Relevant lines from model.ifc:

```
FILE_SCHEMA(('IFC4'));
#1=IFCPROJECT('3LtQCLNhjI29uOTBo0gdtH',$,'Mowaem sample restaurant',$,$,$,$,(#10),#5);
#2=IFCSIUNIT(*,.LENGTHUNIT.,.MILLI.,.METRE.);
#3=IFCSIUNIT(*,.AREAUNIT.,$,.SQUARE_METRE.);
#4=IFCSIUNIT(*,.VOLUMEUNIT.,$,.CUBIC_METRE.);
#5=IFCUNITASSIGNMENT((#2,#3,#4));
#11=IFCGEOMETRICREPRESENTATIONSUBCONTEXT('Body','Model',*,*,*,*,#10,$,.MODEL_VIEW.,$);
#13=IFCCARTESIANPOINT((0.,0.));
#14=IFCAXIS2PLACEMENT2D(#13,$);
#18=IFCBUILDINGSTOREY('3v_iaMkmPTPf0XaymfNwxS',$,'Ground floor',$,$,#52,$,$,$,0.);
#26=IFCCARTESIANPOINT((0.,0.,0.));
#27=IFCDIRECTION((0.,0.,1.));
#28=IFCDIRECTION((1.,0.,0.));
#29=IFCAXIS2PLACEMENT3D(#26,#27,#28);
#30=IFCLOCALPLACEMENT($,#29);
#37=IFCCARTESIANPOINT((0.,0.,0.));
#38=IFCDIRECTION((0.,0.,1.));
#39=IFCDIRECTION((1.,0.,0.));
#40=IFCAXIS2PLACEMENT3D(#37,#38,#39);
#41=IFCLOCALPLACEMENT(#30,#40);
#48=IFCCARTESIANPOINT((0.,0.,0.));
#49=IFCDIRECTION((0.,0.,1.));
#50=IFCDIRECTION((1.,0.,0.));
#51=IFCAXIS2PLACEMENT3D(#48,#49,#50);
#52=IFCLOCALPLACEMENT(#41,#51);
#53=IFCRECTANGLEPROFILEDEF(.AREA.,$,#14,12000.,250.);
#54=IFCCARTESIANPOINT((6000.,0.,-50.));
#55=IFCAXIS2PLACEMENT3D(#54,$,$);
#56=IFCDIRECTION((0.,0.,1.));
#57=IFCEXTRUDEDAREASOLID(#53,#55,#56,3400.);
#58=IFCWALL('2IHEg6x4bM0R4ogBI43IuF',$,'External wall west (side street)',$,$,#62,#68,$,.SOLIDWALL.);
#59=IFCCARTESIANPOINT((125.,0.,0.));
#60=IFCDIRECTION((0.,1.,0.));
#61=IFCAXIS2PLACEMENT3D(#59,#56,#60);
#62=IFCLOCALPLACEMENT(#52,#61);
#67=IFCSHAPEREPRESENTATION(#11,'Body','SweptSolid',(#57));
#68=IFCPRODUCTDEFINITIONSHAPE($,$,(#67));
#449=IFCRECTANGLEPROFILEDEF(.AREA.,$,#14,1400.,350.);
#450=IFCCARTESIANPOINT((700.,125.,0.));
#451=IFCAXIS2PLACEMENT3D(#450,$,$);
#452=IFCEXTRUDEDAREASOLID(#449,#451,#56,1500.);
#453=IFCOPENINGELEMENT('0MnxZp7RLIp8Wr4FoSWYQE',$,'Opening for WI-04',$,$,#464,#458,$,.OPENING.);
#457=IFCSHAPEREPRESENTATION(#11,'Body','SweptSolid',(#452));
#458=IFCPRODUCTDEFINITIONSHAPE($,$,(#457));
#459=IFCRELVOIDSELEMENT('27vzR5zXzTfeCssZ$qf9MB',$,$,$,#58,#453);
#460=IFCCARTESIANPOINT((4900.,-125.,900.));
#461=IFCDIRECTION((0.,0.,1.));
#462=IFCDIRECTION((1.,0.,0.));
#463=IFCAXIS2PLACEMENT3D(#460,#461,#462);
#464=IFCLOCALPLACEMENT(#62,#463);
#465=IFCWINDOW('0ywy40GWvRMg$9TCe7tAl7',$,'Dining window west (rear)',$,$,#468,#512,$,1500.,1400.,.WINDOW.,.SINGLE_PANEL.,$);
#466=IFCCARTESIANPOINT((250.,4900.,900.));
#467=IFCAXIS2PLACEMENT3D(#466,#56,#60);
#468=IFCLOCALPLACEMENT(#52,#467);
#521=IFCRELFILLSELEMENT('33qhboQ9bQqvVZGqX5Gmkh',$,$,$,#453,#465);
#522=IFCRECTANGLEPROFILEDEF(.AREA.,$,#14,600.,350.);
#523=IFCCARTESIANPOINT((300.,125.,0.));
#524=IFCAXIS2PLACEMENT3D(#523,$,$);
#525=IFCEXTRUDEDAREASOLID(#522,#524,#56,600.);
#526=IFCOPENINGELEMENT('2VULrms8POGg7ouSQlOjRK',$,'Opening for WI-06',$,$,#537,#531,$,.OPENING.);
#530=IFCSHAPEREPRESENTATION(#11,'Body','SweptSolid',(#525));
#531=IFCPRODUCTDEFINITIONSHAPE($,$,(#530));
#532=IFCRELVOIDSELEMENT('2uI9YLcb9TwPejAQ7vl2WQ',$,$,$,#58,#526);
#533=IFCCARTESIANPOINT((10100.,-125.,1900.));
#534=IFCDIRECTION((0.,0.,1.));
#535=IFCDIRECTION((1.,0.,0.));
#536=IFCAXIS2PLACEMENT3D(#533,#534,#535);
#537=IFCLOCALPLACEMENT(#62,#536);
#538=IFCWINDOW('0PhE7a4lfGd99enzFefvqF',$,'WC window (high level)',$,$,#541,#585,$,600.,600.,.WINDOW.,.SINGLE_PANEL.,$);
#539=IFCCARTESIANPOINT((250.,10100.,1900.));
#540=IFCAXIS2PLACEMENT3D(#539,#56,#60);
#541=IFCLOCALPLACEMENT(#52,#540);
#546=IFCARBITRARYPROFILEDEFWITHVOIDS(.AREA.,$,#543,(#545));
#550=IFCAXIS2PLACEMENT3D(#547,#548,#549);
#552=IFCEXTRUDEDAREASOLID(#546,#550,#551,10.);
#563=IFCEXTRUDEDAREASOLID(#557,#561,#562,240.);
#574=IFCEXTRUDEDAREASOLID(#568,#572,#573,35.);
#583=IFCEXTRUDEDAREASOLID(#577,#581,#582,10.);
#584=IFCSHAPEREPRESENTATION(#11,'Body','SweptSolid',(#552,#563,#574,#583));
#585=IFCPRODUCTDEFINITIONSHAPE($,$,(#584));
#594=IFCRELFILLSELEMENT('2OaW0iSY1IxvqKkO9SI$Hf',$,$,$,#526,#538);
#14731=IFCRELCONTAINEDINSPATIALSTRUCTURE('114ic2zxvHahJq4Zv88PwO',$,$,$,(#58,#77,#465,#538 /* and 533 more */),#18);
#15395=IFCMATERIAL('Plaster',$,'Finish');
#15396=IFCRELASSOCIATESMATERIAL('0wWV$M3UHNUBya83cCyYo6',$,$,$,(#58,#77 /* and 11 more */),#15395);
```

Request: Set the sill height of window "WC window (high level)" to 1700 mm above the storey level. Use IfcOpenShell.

```python
import numpy as np
import ifcopenshell
import ifcopenshell.api.geometry
import ifcopenshell.geom
import ifcopenshell.util.element
import ifcopenshell.util.placement
import ifcopenshell.util.shape
import ifcopenshell.util.unit

model = ifcopenshell.open("model.ifc")
unit_scale = ifcopenshell.util.unit.calculate_unit_scale(model)

window = model.by_guid("0PhE7a4lfGd99enzFefvqF")
opening = window.FillsVoids[0].RelatingOpeningElement
storey = ifcopenshell.util.element.get_container(window, ifc_class="IfcBuildingStorey")
level = ifcopenshell.util.placement.get_local_placement(storey.ObjectPlacement)[2, 3]

# The opening's origin need not be at the sill, so measure its lowest point.
shape = ifcopenshell.geom.create_shape(ifcopenshell.geom.settings(), opening)
bottom = ifcopenshell.util.shape.get_shape_bottom_elevation(shape, shape.geometry) / unit_scale
dz = level + 1.7 / unit_scale - bottom

shift = np.array([0.0, 0.0, dz])
# The window is not placed relative to its opening, so move both.
for product in (opening, window):
    matrix = ifcopenshell.util.placement.get_local_placement(product.ObjectPlacement)
    matrix[:3, 3] += shift
    ifcopenshell.api.geometry.edit_object_placement(model, product=product, matrix=matrix, is_si=False)

print(f"moved by {dz * unit_scale:+.3f} m")

model.write("model-out.ifc")
```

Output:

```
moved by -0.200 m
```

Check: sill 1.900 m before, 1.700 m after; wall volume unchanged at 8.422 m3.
